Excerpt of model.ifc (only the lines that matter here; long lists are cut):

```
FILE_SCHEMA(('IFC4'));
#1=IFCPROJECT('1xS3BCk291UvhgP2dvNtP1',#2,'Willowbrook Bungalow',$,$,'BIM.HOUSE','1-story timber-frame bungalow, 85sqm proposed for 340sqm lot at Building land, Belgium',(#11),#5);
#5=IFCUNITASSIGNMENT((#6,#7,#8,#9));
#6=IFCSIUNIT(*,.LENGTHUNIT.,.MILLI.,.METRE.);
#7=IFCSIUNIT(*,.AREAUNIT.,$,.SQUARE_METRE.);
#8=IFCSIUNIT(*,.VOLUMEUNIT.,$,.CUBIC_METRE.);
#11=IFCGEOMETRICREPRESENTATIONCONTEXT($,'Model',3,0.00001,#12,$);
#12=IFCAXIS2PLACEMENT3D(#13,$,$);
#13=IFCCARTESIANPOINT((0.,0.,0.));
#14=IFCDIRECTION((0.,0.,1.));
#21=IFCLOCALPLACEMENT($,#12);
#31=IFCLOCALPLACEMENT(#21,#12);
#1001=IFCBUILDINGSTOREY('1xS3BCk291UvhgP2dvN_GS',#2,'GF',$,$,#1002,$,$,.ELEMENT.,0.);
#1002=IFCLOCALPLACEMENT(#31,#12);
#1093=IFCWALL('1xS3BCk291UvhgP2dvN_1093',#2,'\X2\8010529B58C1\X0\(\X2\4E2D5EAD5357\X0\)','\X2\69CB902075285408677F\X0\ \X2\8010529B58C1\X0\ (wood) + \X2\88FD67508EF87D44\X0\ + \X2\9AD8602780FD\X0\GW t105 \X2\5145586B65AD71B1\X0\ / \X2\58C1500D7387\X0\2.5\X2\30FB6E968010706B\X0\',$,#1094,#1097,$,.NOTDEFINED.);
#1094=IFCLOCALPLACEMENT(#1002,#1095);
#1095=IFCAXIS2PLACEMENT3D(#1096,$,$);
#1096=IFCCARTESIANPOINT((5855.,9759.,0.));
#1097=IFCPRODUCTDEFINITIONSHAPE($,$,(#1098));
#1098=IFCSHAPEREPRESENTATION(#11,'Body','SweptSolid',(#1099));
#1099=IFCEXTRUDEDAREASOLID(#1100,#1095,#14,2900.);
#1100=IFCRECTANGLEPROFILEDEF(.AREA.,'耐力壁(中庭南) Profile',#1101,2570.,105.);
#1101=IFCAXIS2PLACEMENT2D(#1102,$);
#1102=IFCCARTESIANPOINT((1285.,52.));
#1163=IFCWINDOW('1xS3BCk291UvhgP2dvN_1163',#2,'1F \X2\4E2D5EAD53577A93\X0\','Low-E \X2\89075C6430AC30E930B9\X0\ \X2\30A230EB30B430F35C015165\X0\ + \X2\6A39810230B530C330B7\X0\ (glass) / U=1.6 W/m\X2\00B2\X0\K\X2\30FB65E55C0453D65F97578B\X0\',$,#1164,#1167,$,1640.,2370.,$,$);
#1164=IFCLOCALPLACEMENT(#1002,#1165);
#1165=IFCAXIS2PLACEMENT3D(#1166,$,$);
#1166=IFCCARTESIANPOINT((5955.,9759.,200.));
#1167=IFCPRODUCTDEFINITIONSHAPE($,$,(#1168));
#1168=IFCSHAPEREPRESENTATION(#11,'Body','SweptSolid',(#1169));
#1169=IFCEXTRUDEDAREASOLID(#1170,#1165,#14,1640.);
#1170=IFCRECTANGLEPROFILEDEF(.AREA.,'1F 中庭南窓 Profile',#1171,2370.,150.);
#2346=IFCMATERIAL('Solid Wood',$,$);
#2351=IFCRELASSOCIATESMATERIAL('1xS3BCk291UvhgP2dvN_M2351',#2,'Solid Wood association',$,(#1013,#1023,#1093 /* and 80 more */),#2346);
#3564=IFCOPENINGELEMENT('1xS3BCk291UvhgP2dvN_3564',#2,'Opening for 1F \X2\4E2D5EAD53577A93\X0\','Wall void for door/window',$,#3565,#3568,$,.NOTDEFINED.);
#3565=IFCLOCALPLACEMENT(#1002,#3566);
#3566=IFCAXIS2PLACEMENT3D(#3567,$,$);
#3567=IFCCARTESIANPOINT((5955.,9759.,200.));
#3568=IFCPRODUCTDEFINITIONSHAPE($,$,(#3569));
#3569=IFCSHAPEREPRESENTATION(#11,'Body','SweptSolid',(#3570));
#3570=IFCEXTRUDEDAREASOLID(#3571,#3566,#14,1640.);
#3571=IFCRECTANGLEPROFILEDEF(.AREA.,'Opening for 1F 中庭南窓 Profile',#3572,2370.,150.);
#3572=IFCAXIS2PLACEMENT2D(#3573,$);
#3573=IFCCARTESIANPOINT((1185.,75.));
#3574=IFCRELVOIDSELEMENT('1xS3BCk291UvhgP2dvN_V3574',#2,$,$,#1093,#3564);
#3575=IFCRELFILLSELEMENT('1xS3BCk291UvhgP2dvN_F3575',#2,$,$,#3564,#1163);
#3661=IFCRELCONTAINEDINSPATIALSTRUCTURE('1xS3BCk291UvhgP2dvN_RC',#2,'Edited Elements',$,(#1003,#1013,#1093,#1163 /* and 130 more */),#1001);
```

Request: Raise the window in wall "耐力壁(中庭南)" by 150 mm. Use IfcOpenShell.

```python
import numpy as np
import ifcopenshell
import ifcopenshell.api.geometry
import ifcopenshell.util.placement
import ifcopenshell.util.unit

model = ifcopenshell.open("model.ifc")
unit_scale = ifcopenshell.util.unit.calculate_unit_scale(model)

window = model.by_guid("1xS3BCk291UvhgP2dvN_1163")
opening = window.FillsVoids[0].RelatingOpeningElement
dz = 150.0

shift = np.array([0.0, 0.0, dz])
# The window is not placed relative to its opening, so move both.
for product in (opening, window):
    matrix = ifcopenshell.util.placement.get_local_placement(product.ObjectPlacement)
    matrix[:3, 3] += shift
    ifcopenshell.api.geometry.edit_object_placement(model, product=product, matrix=matrix, is_si=False)

print(f"moved by {dz * unit_scale:+.3f} m")

model.write("model_updated.ifc")
```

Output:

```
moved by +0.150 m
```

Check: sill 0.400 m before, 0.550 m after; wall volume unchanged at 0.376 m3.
